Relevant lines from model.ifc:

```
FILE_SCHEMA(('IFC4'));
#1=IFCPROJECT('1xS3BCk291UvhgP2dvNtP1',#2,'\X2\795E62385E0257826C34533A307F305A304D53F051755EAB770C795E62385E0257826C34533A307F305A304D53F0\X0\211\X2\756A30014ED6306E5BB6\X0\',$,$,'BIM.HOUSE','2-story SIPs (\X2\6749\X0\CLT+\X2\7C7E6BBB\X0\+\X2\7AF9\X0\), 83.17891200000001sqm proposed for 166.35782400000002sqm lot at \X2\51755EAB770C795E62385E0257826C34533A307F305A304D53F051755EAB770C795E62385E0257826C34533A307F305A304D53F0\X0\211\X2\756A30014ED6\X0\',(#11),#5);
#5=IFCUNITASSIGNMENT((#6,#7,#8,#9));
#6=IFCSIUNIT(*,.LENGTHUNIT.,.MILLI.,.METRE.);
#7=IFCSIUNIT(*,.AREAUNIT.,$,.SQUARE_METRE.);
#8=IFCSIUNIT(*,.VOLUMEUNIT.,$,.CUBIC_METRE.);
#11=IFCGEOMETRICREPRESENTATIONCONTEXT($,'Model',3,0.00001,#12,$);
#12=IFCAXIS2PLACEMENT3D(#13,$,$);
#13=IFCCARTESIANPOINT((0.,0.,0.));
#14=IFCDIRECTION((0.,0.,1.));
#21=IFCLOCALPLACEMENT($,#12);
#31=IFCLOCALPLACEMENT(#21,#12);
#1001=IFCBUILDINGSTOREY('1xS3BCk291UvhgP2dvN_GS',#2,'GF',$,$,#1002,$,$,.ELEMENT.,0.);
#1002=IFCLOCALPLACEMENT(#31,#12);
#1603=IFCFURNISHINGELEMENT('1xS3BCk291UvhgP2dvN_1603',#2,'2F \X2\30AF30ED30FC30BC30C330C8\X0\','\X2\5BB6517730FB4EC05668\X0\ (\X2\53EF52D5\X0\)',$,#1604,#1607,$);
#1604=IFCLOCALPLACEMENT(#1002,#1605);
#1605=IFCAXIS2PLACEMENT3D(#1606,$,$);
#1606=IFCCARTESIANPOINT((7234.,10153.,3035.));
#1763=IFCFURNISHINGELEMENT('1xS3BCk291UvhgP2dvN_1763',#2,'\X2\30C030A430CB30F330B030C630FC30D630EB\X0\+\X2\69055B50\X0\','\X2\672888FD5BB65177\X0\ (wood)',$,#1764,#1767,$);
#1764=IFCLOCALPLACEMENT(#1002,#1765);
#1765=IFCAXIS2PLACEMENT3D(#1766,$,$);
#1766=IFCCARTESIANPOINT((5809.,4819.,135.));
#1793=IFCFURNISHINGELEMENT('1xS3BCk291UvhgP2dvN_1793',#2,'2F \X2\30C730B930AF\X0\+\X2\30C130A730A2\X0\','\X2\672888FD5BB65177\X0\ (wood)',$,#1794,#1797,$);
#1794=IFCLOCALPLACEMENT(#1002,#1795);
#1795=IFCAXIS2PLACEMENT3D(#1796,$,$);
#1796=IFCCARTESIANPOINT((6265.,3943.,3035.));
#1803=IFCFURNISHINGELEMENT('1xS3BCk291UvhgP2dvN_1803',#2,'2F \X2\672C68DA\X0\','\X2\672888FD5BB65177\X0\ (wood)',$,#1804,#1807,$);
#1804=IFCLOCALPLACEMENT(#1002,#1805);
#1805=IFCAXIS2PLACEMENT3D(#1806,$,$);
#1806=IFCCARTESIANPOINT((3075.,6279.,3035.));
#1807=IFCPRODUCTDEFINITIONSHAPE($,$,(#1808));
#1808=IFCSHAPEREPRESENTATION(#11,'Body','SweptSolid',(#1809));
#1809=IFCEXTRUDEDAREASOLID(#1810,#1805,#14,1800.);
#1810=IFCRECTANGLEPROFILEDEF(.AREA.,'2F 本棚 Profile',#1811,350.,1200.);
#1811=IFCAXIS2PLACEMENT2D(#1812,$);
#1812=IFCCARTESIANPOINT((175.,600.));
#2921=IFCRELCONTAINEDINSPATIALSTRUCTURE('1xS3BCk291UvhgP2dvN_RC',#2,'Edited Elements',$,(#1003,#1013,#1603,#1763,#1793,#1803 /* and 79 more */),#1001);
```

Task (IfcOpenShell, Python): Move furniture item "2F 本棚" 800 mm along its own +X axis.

```python
import ifcopenshell
import ifcopenshell.api.geometry
import ifcopenshell.util.placement

model = ifcopenshell.open("model.ifc")

item = model.by_id(1803)
matrix = ifcopenshell.util.placement.get_local_placement(item.ObjectPlacement)
matrix[:3, 3] += matrix[:3, 0] * 800.0
ifcopenshell.api.geometry.edit_object_placement(model, product=item, matrix=matrix, is_si=False)

print(ifcopenshell.util.placement.get_local_placement(item.ObjectPlacement).round(3) + 0.0)

model.write("model_edited.ifc")
```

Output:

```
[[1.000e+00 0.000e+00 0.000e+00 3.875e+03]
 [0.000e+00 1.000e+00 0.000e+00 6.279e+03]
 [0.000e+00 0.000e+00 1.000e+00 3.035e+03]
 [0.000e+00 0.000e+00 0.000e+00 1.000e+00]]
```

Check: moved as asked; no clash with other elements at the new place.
